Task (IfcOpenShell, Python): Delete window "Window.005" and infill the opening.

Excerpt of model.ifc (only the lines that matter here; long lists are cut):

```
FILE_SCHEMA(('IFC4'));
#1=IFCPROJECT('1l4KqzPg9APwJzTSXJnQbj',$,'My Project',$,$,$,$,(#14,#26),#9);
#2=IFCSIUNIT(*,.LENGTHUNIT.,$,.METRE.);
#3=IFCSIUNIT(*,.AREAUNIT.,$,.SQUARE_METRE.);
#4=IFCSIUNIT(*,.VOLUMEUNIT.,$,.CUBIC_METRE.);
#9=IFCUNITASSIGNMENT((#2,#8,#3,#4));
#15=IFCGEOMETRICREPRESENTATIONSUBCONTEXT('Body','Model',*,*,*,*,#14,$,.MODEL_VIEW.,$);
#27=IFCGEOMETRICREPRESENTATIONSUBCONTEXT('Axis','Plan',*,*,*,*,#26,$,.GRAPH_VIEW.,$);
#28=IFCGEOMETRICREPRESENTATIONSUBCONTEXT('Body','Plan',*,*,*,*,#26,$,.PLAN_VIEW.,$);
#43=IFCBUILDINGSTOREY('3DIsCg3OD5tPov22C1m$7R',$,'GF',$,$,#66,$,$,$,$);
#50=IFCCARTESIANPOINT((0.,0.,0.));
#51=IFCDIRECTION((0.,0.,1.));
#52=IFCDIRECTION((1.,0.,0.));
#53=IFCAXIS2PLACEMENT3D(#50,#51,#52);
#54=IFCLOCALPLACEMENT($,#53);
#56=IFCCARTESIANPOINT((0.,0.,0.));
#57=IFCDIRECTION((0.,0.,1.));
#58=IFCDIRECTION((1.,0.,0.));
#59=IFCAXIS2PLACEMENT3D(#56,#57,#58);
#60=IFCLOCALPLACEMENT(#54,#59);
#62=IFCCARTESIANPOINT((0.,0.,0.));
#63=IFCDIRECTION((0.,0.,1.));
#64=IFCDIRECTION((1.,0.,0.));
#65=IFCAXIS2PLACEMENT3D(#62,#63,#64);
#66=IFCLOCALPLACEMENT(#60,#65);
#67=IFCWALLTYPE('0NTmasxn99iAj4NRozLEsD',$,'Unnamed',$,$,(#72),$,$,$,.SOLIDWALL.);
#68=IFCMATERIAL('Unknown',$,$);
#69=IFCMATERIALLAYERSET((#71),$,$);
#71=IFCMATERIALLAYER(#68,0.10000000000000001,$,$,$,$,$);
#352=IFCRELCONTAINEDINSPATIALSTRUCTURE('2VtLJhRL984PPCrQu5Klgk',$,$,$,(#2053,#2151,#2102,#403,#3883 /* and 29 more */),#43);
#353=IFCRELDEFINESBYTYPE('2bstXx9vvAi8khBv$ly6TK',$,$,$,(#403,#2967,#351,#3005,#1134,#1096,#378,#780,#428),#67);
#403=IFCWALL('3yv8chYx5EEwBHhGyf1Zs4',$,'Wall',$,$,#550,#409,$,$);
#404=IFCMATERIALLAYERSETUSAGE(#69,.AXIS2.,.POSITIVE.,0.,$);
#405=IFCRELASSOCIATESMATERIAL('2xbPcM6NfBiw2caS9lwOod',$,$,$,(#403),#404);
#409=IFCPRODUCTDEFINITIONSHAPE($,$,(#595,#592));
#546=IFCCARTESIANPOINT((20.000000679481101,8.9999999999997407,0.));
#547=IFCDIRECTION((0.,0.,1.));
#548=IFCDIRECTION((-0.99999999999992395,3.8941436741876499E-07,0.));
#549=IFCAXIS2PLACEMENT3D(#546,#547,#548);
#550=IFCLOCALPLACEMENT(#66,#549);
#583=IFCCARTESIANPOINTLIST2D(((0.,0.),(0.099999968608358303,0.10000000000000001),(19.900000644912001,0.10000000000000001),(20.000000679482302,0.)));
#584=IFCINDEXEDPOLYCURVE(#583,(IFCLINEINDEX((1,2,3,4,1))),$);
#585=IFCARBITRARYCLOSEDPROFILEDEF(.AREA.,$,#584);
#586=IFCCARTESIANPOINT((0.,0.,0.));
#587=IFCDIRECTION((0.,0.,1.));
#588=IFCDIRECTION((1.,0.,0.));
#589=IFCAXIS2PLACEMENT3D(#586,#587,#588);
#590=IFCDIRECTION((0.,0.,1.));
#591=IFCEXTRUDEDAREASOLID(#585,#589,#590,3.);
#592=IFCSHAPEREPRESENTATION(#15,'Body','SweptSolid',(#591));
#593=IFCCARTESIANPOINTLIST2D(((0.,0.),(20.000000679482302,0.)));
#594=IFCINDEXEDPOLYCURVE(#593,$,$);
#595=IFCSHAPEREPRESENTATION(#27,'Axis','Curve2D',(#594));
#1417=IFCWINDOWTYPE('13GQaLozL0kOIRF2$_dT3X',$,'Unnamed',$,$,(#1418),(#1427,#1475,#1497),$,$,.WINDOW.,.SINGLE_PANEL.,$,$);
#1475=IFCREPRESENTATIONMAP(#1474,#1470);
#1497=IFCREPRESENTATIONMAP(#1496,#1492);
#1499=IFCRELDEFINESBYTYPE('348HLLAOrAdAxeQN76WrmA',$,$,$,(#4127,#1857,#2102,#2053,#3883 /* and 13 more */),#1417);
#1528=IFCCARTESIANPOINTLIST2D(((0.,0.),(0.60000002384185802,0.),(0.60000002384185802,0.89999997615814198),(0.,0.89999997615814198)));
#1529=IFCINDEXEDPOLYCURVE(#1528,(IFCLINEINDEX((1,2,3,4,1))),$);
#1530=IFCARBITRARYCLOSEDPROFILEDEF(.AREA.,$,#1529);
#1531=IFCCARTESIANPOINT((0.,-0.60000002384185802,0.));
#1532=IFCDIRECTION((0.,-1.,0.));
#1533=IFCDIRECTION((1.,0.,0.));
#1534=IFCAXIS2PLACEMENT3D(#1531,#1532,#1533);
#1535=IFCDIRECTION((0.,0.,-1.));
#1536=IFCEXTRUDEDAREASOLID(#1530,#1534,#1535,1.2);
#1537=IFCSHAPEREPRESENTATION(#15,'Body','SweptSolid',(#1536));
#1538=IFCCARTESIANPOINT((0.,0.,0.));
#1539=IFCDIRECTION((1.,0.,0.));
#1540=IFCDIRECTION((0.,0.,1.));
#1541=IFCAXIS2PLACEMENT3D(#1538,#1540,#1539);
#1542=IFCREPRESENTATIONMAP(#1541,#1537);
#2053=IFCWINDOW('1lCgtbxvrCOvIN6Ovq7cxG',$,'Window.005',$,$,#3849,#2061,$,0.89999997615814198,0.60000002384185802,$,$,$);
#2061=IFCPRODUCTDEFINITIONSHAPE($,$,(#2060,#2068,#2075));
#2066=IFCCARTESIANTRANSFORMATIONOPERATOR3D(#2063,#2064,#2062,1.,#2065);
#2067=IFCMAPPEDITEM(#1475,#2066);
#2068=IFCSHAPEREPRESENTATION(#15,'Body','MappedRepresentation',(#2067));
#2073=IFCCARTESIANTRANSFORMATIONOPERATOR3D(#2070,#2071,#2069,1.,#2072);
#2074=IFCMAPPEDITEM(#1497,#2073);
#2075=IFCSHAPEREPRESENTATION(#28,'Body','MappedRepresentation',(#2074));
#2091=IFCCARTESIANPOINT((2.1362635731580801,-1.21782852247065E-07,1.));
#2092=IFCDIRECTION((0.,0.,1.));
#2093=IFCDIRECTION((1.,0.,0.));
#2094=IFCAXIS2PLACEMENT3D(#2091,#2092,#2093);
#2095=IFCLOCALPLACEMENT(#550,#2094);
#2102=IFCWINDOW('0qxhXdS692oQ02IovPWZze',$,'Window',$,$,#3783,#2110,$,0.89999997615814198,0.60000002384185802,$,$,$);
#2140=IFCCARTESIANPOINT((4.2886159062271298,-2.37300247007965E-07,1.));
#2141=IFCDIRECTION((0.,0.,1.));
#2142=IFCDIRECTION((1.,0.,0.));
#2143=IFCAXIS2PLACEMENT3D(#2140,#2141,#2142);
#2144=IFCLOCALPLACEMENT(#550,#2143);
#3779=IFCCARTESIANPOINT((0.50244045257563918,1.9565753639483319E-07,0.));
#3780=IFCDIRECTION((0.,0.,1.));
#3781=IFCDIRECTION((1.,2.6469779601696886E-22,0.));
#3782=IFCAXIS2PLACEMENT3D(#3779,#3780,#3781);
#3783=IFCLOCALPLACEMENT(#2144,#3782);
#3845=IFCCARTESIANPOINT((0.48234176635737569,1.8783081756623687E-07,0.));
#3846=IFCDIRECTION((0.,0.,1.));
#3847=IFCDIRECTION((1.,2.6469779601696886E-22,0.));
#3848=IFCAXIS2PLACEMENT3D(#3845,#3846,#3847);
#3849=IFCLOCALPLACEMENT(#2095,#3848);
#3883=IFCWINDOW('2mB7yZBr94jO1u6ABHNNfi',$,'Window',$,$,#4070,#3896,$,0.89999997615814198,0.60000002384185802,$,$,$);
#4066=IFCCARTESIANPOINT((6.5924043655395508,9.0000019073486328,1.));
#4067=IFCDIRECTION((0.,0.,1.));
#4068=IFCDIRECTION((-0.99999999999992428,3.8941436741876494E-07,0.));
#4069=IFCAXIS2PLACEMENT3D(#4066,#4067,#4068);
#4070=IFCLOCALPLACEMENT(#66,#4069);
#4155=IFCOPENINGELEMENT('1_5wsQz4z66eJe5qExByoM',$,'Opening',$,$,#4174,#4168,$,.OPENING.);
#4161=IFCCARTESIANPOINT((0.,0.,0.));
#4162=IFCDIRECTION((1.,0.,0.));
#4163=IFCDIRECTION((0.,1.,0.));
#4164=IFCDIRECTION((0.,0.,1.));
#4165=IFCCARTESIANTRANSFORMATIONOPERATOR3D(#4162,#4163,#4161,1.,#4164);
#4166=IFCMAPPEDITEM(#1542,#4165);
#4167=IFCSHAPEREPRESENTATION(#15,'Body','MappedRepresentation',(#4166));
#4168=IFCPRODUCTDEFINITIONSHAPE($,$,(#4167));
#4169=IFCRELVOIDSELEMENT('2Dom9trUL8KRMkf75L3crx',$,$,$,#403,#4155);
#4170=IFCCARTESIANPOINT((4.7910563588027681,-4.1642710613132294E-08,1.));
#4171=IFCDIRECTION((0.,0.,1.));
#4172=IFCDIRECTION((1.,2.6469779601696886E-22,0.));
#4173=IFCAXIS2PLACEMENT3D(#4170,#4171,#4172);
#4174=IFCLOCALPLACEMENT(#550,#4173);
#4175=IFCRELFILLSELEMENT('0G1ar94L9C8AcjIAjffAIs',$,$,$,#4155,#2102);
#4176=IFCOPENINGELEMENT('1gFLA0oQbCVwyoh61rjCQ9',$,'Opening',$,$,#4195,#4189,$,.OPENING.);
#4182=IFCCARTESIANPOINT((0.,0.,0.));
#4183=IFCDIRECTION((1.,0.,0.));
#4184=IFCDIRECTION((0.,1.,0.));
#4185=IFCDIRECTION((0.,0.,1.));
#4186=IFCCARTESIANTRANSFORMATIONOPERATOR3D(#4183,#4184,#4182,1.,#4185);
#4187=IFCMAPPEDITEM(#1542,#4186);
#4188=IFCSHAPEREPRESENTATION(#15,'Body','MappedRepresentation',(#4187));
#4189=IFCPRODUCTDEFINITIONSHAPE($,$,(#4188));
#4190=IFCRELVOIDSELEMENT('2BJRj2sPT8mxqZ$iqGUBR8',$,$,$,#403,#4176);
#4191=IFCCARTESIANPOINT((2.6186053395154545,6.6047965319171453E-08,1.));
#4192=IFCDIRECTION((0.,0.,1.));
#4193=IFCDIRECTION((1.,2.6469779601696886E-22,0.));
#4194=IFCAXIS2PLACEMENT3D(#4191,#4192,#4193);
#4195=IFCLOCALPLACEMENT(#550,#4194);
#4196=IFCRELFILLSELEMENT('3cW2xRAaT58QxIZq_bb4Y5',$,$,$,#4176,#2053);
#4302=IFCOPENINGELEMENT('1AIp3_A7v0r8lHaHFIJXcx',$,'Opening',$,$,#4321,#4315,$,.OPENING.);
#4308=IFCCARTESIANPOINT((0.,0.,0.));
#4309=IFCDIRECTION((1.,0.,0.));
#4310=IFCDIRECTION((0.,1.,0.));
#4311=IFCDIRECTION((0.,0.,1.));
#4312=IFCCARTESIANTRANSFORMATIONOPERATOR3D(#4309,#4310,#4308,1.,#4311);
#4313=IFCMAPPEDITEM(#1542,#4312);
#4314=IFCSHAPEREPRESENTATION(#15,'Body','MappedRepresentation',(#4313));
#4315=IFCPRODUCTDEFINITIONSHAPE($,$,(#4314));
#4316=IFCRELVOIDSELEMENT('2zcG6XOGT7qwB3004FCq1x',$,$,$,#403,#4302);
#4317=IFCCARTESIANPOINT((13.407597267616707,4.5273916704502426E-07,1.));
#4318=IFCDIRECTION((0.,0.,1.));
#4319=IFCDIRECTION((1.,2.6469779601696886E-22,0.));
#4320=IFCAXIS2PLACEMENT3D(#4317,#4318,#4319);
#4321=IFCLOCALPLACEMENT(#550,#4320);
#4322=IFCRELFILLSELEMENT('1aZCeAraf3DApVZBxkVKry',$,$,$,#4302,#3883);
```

```python
import ifcopenshell
import ifcopenshell.api.feature
import ifcopenshell.api.root
import ifcopenshell.geom
import ifcopenshell.util.shape

model = ifcopenshell.open("model.ifc")
settings = ifcopenshell.geom.settings()


def volume(element):
    """Net volume in cubic metres, openings subtracted."""
    shape = ifcopenshell.geom.create_shape(settings, element)
    return ifcopenshell.util.shape.get_volume(shape.geometry)


window = model.by_guid("1lCgtbxvrCOvIN6Ovq7cxG")
opening = window.FillsVoids[0].RelatingOpeningElement
wall = opening.VoidsElements[0].RelatingBuildingElement
before = volume(wall)

ifcopenshell.api.root.remove_product(model, product=window)
ifcopenshell.api.feature.remove_feature(model, feature=opening)

after = volume(wall)

print(f"wall volume {before:.3f} -> {after:.3f} m3")

model.write("model_rev.ifc")
```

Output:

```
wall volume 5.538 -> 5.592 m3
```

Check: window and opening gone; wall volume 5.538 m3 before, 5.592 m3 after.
